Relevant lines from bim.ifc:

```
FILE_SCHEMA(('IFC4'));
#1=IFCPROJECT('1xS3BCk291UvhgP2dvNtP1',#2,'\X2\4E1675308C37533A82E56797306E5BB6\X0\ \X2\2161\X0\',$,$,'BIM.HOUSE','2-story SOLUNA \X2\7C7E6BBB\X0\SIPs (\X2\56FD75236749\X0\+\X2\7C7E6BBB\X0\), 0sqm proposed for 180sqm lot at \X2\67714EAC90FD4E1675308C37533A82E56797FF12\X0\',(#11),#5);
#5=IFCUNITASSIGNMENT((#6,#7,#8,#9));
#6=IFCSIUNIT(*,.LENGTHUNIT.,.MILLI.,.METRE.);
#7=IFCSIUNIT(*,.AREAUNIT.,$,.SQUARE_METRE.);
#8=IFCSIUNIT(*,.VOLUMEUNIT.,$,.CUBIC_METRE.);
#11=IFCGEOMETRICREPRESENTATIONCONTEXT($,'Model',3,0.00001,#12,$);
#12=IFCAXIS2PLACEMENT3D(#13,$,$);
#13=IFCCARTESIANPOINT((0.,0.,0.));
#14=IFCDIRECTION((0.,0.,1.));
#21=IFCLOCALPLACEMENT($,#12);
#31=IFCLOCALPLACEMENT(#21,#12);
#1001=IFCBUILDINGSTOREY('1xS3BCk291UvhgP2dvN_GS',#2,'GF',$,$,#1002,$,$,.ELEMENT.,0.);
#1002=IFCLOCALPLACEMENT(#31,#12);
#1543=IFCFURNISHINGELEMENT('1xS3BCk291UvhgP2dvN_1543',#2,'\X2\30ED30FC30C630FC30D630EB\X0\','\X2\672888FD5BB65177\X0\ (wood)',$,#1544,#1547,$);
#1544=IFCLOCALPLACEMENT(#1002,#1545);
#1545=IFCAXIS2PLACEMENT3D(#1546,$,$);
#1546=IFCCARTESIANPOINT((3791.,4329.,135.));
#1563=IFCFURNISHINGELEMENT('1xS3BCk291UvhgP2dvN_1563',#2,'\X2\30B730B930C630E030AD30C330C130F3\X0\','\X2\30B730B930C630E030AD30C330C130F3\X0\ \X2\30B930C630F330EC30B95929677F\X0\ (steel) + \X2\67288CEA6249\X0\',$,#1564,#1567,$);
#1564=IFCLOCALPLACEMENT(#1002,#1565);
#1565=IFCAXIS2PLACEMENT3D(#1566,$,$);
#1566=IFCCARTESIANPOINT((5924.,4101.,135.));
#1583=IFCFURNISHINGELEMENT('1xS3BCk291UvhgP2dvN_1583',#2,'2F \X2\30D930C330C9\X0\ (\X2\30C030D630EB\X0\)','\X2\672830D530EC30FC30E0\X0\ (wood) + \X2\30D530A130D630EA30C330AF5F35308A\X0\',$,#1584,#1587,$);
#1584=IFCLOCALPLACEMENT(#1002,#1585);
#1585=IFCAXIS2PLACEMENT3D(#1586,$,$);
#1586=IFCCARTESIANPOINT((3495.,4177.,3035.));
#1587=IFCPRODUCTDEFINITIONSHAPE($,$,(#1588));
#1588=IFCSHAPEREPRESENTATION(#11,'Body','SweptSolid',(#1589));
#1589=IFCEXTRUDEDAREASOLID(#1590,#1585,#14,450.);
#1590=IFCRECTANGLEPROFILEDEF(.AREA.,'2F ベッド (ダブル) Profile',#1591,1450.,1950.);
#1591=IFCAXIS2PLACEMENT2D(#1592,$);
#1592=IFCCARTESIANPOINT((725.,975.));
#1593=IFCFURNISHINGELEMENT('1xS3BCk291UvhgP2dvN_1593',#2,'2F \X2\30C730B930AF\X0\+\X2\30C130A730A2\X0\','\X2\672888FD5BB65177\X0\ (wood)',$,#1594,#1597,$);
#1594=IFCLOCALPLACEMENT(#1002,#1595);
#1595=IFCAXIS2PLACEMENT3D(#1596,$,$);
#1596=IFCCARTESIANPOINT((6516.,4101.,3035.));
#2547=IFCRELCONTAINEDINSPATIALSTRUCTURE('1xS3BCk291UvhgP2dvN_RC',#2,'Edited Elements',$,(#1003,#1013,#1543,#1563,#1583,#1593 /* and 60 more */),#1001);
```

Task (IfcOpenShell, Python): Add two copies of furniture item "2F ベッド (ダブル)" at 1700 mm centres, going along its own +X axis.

```python
import ifcopenshell
import ifcopenshell.api.geometry
import ifcopenshell.api.root
import ifcopenshell.util.element
import ifcopenshell.util.placement

model = ifcopenshell.open("bim.ifc")


def reuse_history(source, copy):
    """copy_class also copies each property set's owner history, people and application; keep the originals."""
    for rel in copy.IsDefinedBy:
        if rel.is_a("IfcRelDefinesByProperties") and (history := rel.RelatingPropertyDefinition.OwnerHistory):
            rel.RelatingPropertyDefinition.OwnerHistory = source.OwnerHistory
            ifcopenshell.util.element.remove_deep2(model, history)


source = model.by_guid("1xS3BCk291UvhgP2dvN_1583")
base = ifcopenshell.util.placement.get_local_placement(source.ObjectPlacement)
step = base[:3, 0] * 1700.0

for i in range(1, 3):
    copy = ifcopenshell.api.root.copy_class(model, product=source)
    copy.Representation = ifcopenshell.util.element.copy_deep(
        model, source.Representation, exclude=["IfcGeometricRepresentationContext", "IfcRepresentationMap"]
    )
    reuse_history(source, copy)
    matrix = base.copy()
    matrix[:3, 3] += i * step
    print("added at", matrix[:3, 3].round(3) + 0.0)
    ifcopenshell.api.geometry.edit_object_placement(model, product=copy, matrix=matrix, is_si=False)

model.write("bim_v2.ifc")
```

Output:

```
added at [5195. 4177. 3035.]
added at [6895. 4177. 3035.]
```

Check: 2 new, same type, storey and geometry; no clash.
